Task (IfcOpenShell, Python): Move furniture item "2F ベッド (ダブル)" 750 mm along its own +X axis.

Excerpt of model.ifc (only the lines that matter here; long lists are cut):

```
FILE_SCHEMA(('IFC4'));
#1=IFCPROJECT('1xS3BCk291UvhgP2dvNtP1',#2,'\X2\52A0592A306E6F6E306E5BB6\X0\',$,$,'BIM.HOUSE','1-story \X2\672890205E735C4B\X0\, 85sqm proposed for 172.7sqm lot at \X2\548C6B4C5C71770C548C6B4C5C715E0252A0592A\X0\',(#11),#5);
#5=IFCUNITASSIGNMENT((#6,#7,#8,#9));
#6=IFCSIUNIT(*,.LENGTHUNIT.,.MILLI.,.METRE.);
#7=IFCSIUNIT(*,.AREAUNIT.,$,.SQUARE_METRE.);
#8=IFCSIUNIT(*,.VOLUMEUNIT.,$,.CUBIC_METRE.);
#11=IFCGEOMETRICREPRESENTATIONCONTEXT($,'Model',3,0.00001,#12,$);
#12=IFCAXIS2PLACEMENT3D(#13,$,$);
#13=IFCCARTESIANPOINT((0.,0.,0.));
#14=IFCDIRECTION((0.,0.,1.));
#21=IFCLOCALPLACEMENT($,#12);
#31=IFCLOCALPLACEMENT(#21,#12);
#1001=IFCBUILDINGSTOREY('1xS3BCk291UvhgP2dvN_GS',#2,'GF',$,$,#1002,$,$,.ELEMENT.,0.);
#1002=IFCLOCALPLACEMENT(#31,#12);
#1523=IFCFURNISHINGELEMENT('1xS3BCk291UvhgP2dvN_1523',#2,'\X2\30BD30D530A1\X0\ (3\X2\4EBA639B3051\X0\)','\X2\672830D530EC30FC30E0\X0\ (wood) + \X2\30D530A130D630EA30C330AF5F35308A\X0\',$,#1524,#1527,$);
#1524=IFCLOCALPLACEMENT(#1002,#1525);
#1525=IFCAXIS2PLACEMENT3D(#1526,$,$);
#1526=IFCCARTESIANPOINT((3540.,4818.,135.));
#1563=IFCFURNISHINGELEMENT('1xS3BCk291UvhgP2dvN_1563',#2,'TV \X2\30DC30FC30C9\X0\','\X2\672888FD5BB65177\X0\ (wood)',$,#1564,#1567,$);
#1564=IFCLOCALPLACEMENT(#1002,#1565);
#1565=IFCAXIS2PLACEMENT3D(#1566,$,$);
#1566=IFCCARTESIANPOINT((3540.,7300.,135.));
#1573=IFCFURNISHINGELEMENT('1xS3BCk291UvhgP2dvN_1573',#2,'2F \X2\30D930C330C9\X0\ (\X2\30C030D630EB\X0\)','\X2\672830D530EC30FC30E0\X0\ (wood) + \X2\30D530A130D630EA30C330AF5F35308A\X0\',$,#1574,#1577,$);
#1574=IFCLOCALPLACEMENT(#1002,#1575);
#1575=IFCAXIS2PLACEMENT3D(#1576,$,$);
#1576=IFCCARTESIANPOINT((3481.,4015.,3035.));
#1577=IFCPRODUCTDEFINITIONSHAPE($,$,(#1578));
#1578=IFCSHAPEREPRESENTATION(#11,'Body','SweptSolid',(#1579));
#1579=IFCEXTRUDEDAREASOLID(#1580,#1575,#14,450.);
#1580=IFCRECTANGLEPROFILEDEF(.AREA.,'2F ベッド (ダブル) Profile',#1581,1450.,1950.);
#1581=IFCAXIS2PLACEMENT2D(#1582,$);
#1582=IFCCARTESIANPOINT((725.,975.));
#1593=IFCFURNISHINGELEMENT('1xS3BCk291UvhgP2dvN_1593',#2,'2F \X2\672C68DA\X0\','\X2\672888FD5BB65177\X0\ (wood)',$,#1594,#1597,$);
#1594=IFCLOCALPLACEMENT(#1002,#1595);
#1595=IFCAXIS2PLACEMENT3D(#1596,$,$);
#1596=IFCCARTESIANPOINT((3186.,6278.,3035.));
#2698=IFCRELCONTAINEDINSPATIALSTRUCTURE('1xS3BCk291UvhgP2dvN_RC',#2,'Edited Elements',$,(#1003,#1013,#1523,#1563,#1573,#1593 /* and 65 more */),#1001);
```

```python
import ifcopenshell
import ifcopenshell.api.geometry
import ifcopenshell.util.placement
import ifcopenshell.util.unit

model = ifcopenshell.open("model.ifc")
unit_scale = ifcopenshell.util.unit.calculate_unit_scale(model)

item = model.by_guid("1xS3BCk291UvhgP2dvN_1573")
matrix = ifcopenshell.util.placement.get_local_placement(item.ObjectPlacement)
matrix[:3, 3] += matrix[:3, 0] * 0.75 / unit_scale
ifcopenshell.api.geometry.edit_object_placement(model, product=item, matrix=matrix, is_si=False)

print(ifcopenshell.util.placement.get_local_placement(item.ObjectPlacement).round(3) + 0.0)

model.write("model_edited.ifc")
```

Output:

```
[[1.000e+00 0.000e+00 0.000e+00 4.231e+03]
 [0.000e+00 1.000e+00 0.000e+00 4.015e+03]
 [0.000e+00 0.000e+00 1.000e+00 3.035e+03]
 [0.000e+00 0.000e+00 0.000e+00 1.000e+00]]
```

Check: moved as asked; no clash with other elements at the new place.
